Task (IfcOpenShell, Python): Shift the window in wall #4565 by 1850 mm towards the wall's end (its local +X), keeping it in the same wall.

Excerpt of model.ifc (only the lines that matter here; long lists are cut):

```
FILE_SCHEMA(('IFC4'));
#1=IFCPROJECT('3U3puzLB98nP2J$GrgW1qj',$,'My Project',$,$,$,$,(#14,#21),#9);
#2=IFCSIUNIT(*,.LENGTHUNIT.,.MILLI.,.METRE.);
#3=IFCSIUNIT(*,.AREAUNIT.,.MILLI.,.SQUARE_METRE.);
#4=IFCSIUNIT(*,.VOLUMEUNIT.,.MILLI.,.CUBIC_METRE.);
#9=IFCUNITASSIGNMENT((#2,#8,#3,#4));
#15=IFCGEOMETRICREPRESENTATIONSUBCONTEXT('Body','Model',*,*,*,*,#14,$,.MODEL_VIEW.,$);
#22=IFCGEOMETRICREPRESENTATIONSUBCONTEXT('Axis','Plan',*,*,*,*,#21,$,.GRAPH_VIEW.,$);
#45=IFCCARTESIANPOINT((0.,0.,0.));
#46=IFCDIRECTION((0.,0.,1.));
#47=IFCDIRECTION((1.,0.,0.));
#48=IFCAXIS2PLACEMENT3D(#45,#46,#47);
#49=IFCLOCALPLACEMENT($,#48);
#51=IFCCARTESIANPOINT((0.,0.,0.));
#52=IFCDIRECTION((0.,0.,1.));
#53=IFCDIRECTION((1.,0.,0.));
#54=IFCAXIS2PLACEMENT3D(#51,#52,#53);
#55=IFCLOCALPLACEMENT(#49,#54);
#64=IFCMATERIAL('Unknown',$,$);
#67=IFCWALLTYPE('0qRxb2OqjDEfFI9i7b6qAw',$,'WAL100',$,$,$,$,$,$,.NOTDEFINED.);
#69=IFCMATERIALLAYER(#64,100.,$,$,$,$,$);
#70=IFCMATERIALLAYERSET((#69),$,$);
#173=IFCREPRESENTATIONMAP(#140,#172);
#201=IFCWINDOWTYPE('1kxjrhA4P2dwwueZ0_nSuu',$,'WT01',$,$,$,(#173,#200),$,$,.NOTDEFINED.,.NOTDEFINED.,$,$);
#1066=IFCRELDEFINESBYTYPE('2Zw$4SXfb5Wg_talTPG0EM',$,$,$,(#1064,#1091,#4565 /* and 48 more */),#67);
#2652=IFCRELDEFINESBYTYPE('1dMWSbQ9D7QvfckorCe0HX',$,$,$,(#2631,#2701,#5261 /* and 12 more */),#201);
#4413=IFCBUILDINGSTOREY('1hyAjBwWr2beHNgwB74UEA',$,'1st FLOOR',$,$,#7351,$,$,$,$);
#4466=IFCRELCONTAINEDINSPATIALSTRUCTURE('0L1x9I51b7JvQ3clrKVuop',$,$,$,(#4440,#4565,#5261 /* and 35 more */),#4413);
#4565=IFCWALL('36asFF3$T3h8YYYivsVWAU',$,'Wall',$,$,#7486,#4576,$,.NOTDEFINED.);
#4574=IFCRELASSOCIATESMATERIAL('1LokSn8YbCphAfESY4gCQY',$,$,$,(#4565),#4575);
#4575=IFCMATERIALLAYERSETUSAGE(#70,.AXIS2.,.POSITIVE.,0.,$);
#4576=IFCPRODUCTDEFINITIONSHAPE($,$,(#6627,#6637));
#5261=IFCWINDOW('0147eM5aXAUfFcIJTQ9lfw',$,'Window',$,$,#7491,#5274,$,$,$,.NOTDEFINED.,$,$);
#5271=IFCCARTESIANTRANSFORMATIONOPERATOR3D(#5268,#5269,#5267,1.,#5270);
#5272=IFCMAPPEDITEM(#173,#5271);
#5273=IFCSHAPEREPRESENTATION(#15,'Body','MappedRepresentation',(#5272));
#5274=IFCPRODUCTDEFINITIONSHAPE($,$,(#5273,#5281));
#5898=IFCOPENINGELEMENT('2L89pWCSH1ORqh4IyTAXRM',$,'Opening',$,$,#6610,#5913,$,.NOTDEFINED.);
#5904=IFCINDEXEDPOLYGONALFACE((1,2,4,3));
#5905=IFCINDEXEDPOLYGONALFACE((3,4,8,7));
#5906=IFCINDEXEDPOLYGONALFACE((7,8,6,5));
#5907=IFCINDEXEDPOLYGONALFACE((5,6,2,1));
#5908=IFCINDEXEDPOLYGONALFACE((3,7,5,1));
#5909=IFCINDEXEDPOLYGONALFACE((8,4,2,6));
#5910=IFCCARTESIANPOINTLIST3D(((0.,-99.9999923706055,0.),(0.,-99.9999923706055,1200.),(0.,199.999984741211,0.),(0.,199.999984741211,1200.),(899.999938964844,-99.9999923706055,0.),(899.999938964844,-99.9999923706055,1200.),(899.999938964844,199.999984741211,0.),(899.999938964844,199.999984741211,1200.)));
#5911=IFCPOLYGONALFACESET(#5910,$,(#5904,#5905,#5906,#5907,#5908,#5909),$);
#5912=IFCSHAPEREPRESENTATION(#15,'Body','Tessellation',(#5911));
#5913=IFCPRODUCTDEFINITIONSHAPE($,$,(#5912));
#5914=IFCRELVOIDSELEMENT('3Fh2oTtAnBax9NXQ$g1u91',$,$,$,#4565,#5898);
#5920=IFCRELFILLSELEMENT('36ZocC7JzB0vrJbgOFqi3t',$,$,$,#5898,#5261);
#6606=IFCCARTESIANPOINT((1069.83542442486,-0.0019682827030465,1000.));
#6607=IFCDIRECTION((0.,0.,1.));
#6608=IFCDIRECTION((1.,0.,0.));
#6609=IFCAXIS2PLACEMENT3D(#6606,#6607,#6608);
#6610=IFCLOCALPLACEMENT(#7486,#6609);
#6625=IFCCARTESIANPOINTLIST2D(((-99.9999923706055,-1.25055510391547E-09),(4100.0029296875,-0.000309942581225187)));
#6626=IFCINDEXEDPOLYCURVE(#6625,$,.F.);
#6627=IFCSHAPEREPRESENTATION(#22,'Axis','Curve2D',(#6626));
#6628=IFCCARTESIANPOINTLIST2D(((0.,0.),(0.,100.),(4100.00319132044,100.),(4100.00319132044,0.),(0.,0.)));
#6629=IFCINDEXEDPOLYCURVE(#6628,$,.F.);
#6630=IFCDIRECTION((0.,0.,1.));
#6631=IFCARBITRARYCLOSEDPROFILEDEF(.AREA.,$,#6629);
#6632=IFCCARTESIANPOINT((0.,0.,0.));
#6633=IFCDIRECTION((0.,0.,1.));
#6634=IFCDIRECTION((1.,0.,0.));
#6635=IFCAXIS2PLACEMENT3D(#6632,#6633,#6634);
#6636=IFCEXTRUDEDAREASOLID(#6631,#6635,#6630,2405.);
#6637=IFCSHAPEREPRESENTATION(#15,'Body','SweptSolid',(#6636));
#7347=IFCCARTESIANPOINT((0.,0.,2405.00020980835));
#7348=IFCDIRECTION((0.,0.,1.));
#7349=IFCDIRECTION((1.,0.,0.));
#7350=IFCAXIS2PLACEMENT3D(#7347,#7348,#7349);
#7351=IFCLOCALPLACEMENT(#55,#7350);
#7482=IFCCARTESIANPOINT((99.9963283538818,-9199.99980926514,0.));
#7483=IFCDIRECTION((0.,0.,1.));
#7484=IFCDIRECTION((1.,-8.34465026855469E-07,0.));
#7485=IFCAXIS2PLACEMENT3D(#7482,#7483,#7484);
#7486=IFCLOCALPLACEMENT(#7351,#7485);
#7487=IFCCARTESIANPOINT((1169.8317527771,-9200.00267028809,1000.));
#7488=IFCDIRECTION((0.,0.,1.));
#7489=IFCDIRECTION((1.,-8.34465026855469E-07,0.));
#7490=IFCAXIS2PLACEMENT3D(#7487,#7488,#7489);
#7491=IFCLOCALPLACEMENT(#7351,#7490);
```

```python
import ifcopenshell
import ifcopenshell.api.geometry
import ifcopenshell.util.placement
import ifcopenshell.util.unit

model = ifcopenshell.open("model.ifc")
unit_scale = ifcopenshell.util.unit.calculate_unit_scale(model)

window = model.by_id(5261)
opening = window.FillsVoids[0].RelatingOpeningElement
wall = opening.VoidsElements[0].RelatingBuildingElement

wall_matrix = ifcopenshell.util.placement.get_local_placement(wall.ObjectPlacement)
shift = wall_matrix[:3, 0] * 1.85 / unit_scale
before = ifcopenshell.util.placement.get_local_placement(window.ObjectPlacement)[:3, 3].copy()

# The window is not placed relative to its opening, so move both.
for product in (opening, window):
    matrix = ifcopenshell.util.placement.get_local_placement(product.ObjectPlacement)
    matrix[:3, 3] += shift
    ifcopenshell.api.geometry.edit_object_placement(model, product=product, matrix=matrix, is_si=False)

after = ifcopenshell.util.placement.get_local_placement(window.ObjectPlacement)[:3, 3]
print("window moved by", (after - before).round(3) + 0.0)

model.write("model_updated.ifc")
```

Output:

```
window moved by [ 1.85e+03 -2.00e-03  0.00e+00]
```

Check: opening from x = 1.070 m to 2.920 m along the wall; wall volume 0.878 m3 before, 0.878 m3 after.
